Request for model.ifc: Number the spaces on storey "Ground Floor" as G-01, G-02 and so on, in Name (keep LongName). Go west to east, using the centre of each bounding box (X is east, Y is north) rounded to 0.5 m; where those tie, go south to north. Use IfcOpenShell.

First a look at what the model holds.

```python
import ifcopenshell
import ifcopenshell.util.element
import ifcopenshell.util.placement

model = ifcopenshell.open("model.ifc")
print(model.schema)
storey = next(s for s in model.by_type("IfcBuildingStorey") if s.Name == "Ground Floor")
spaces = [e for e in ifcopenshell.util.element.get_decomposition(storey) if e.is_a("IfcSpace")]
for e in sorted(spaces, key=lambda e: e.id()):
    origin = ifcopenshell.util.placement.get_local_placement(e.ObjectPlacement)[:3, 3]
    print(e.id(), e.Name, e.LongName, origin.round(2) + 0.0, sep=" | ")
```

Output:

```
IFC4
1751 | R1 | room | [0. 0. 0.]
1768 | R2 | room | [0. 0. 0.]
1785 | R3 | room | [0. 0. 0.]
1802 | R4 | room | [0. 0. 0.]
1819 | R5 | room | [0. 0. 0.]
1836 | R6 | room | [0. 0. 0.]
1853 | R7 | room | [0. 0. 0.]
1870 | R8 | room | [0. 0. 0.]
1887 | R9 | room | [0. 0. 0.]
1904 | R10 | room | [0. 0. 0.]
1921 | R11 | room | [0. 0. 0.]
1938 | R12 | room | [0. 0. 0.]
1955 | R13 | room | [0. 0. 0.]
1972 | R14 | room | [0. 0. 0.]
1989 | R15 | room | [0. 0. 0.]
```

```python
import ifcopenshell
import ifcopenshell.geom
import ifcopenshell.util.element
import ifcopenshell.util.shape

model = ifcopenshell.open("model.ifc")
settings = ifcopenshell.geom.settings()
settings.set("use-world-coords", True)


def centre(element):
    shape = ifcopenshell.geom.create_shape(settings, element)
    return ifcopenshell.util.shape.get_bbox_centroid(shape.geometry)


storey = next(s for s in model.by_type("IfcBuildingStorey") if s.Name == "Ground Floor")
spaces = [e for e in ifcopenshell.util.element.get_decomposition(storey) if e.is_a("IfcSpace")]

# Insertion points can sit at a corner or the storey origin, so sort by the geometry (in metres).
centres = {e: centre(e) for e in spaces}
spaces.sort(key=lambda e: (round(centres[e][0] / 0.5), centres[e][1]))

for i, e in enumerate(spaces, start=1):
    number = f"G-{i:02d}"
    e.Name = number
    print(e.id(), number)

model.write("model_updated.ifc")
```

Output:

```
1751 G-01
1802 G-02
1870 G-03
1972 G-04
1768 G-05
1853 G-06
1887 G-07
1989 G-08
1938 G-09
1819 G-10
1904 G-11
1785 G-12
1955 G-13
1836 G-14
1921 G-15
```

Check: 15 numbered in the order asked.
